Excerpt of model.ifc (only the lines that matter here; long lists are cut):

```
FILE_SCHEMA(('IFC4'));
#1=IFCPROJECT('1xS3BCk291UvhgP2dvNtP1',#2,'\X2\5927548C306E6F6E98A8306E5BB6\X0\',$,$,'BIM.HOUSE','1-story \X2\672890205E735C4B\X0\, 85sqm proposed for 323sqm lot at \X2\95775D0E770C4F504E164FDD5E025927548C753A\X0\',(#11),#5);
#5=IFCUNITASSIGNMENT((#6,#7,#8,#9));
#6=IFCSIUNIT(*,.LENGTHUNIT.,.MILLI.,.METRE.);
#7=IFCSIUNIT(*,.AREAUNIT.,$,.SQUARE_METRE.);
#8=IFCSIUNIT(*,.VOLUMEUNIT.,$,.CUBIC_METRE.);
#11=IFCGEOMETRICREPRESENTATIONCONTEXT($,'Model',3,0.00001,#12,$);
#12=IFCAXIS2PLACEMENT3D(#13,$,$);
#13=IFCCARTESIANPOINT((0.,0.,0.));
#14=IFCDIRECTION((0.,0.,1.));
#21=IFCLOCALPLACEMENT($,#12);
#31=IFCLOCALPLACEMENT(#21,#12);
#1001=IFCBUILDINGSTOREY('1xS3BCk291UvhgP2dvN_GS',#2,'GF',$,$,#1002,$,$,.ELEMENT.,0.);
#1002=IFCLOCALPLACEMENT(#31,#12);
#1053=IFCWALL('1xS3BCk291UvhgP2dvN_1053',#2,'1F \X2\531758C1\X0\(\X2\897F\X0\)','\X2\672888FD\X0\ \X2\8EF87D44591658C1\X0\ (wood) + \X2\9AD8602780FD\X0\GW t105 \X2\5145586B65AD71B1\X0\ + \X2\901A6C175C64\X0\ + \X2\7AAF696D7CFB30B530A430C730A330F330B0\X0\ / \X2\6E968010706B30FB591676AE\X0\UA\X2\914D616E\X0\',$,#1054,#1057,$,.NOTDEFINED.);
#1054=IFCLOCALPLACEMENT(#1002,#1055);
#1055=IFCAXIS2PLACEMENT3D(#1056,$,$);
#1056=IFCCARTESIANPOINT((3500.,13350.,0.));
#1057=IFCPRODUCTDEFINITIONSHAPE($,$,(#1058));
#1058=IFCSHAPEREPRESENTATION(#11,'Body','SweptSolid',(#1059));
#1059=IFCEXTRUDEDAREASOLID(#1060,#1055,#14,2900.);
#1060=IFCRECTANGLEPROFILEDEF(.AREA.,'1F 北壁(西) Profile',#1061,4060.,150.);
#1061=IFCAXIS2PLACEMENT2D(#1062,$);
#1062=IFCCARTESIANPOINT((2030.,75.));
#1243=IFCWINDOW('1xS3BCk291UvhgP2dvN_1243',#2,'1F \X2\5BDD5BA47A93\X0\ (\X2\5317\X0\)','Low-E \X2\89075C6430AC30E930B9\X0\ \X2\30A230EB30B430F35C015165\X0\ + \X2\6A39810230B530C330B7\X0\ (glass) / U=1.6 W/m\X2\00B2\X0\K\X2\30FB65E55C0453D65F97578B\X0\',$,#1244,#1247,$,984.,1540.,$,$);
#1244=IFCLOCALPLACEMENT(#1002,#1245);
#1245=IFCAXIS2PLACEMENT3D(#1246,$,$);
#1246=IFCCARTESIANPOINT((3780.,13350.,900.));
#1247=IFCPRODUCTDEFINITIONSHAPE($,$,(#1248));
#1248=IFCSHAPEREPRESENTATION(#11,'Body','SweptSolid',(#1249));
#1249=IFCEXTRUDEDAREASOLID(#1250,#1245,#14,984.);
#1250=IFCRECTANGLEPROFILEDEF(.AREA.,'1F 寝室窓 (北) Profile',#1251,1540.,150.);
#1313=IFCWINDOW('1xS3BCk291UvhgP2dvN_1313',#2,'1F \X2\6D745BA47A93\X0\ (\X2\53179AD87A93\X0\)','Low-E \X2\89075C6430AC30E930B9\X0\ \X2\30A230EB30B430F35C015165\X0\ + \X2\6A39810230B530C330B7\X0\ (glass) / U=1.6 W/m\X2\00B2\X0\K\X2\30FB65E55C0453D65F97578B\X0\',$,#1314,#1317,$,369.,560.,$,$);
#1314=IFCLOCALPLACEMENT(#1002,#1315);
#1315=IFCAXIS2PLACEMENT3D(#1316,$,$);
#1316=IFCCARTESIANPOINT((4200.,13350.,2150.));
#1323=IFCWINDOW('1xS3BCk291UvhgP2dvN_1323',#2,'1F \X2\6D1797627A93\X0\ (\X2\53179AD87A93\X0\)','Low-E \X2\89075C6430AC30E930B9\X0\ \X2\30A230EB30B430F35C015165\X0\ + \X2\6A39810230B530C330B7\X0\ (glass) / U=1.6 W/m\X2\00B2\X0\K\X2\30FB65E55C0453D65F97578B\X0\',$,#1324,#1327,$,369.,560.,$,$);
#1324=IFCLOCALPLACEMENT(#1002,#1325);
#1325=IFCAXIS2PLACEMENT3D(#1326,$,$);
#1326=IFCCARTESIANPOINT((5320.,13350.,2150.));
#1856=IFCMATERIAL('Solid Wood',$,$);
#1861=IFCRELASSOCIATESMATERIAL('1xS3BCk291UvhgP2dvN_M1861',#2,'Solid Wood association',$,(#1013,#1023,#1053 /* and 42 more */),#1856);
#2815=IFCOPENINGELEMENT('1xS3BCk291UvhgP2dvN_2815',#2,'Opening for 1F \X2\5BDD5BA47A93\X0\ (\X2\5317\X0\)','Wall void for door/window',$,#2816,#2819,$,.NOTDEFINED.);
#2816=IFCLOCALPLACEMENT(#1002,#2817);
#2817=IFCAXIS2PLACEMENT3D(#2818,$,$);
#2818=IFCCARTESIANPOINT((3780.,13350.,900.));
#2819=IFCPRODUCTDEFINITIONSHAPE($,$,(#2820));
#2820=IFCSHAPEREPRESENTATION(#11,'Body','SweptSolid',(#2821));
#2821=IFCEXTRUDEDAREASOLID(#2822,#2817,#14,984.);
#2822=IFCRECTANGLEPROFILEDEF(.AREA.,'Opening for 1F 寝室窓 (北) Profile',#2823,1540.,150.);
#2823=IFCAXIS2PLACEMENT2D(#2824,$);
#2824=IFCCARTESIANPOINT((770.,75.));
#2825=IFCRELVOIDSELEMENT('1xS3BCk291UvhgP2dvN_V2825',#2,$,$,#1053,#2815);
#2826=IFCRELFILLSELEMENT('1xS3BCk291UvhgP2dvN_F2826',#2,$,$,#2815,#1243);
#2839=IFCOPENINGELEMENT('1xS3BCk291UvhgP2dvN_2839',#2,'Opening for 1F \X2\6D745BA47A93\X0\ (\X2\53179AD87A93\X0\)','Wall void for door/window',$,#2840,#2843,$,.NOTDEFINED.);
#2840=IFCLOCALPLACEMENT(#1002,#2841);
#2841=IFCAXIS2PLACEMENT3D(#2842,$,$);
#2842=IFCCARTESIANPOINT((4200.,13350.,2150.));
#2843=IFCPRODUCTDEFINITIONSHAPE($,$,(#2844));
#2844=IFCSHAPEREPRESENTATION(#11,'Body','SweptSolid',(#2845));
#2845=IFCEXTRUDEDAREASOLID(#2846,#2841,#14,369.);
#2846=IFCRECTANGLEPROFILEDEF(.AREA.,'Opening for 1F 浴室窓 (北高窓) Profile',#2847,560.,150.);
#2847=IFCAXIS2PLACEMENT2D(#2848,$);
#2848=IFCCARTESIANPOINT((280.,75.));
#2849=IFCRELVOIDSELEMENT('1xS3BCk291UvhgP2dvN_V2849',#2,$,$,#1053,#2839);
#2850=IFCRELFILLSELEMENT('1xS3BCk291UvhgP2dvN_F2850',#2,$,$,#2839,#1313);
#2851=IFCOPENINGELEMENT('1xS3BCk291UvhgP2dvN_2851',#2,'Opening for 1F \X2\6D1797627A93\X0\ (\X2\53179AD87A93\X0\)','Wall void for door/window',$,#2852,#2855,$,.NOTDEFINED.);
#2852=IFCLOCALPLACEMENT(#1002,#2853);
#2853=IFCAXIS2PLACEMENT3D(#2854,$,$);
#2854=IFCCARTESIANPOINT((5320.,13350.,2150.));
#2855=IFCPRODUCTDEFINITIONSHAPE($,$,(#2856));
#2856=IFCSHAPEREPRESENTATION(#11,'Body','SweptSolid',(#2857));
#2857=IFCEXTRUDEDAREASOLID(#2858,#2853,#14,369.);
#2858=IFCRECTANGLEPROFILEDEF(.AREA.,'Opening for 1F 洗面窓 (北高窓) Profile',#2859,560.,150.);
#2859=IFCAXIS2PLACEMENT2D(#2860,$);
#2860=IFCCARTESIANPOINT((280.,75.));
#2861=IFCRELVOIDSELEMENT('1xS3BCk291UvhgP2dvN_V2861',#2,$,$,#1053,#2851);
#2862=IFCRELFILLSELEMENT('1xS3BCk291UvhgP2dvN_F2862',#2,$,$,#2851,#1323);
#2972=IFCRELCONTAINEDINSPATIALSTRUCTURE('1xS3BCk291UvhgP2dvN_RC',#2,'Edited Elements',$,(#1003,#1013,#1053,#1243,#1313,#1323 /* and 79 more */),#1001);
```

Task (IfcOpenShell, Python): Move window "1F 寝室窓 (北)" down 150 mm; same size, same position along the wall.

```python
import numpy as np
import ifcopenshell
import ifcopenshell.api.geometry
import ifcopenshell.util.placement
import ifcopenshell.util.unit

model = ifcopenshell.open("model.ifc")
unit_scale = ifcopenshell.util.unit.calculate_unit_scale(model)

window = model.by_guid("1xS3BCk291UvhgP2dvN_1243")
opening = window.FillsVoids[0].RelatingOpeningElement
dz = -0.15 / unit_scale

shift = np.array([0.0, 0.0, dz])
# The window is not placed relative to its opening, so move both.
for product in (opening, window):
    matrix = ifcopenshell.util.placement.get_local_placement(product.ObjectPlacement)
    matrix[:3, 3] += shift
    ifcopenshell.api.geometry.edit_object_placement(model, product=product, matrix=matrix, is_si=False)

print(f"moved by {dz * unit_scale:+.3f} m")

model.write("model_v2.ifc")
```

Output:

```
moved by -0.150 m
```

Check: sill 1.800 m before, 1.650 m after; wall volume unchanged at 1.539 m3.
